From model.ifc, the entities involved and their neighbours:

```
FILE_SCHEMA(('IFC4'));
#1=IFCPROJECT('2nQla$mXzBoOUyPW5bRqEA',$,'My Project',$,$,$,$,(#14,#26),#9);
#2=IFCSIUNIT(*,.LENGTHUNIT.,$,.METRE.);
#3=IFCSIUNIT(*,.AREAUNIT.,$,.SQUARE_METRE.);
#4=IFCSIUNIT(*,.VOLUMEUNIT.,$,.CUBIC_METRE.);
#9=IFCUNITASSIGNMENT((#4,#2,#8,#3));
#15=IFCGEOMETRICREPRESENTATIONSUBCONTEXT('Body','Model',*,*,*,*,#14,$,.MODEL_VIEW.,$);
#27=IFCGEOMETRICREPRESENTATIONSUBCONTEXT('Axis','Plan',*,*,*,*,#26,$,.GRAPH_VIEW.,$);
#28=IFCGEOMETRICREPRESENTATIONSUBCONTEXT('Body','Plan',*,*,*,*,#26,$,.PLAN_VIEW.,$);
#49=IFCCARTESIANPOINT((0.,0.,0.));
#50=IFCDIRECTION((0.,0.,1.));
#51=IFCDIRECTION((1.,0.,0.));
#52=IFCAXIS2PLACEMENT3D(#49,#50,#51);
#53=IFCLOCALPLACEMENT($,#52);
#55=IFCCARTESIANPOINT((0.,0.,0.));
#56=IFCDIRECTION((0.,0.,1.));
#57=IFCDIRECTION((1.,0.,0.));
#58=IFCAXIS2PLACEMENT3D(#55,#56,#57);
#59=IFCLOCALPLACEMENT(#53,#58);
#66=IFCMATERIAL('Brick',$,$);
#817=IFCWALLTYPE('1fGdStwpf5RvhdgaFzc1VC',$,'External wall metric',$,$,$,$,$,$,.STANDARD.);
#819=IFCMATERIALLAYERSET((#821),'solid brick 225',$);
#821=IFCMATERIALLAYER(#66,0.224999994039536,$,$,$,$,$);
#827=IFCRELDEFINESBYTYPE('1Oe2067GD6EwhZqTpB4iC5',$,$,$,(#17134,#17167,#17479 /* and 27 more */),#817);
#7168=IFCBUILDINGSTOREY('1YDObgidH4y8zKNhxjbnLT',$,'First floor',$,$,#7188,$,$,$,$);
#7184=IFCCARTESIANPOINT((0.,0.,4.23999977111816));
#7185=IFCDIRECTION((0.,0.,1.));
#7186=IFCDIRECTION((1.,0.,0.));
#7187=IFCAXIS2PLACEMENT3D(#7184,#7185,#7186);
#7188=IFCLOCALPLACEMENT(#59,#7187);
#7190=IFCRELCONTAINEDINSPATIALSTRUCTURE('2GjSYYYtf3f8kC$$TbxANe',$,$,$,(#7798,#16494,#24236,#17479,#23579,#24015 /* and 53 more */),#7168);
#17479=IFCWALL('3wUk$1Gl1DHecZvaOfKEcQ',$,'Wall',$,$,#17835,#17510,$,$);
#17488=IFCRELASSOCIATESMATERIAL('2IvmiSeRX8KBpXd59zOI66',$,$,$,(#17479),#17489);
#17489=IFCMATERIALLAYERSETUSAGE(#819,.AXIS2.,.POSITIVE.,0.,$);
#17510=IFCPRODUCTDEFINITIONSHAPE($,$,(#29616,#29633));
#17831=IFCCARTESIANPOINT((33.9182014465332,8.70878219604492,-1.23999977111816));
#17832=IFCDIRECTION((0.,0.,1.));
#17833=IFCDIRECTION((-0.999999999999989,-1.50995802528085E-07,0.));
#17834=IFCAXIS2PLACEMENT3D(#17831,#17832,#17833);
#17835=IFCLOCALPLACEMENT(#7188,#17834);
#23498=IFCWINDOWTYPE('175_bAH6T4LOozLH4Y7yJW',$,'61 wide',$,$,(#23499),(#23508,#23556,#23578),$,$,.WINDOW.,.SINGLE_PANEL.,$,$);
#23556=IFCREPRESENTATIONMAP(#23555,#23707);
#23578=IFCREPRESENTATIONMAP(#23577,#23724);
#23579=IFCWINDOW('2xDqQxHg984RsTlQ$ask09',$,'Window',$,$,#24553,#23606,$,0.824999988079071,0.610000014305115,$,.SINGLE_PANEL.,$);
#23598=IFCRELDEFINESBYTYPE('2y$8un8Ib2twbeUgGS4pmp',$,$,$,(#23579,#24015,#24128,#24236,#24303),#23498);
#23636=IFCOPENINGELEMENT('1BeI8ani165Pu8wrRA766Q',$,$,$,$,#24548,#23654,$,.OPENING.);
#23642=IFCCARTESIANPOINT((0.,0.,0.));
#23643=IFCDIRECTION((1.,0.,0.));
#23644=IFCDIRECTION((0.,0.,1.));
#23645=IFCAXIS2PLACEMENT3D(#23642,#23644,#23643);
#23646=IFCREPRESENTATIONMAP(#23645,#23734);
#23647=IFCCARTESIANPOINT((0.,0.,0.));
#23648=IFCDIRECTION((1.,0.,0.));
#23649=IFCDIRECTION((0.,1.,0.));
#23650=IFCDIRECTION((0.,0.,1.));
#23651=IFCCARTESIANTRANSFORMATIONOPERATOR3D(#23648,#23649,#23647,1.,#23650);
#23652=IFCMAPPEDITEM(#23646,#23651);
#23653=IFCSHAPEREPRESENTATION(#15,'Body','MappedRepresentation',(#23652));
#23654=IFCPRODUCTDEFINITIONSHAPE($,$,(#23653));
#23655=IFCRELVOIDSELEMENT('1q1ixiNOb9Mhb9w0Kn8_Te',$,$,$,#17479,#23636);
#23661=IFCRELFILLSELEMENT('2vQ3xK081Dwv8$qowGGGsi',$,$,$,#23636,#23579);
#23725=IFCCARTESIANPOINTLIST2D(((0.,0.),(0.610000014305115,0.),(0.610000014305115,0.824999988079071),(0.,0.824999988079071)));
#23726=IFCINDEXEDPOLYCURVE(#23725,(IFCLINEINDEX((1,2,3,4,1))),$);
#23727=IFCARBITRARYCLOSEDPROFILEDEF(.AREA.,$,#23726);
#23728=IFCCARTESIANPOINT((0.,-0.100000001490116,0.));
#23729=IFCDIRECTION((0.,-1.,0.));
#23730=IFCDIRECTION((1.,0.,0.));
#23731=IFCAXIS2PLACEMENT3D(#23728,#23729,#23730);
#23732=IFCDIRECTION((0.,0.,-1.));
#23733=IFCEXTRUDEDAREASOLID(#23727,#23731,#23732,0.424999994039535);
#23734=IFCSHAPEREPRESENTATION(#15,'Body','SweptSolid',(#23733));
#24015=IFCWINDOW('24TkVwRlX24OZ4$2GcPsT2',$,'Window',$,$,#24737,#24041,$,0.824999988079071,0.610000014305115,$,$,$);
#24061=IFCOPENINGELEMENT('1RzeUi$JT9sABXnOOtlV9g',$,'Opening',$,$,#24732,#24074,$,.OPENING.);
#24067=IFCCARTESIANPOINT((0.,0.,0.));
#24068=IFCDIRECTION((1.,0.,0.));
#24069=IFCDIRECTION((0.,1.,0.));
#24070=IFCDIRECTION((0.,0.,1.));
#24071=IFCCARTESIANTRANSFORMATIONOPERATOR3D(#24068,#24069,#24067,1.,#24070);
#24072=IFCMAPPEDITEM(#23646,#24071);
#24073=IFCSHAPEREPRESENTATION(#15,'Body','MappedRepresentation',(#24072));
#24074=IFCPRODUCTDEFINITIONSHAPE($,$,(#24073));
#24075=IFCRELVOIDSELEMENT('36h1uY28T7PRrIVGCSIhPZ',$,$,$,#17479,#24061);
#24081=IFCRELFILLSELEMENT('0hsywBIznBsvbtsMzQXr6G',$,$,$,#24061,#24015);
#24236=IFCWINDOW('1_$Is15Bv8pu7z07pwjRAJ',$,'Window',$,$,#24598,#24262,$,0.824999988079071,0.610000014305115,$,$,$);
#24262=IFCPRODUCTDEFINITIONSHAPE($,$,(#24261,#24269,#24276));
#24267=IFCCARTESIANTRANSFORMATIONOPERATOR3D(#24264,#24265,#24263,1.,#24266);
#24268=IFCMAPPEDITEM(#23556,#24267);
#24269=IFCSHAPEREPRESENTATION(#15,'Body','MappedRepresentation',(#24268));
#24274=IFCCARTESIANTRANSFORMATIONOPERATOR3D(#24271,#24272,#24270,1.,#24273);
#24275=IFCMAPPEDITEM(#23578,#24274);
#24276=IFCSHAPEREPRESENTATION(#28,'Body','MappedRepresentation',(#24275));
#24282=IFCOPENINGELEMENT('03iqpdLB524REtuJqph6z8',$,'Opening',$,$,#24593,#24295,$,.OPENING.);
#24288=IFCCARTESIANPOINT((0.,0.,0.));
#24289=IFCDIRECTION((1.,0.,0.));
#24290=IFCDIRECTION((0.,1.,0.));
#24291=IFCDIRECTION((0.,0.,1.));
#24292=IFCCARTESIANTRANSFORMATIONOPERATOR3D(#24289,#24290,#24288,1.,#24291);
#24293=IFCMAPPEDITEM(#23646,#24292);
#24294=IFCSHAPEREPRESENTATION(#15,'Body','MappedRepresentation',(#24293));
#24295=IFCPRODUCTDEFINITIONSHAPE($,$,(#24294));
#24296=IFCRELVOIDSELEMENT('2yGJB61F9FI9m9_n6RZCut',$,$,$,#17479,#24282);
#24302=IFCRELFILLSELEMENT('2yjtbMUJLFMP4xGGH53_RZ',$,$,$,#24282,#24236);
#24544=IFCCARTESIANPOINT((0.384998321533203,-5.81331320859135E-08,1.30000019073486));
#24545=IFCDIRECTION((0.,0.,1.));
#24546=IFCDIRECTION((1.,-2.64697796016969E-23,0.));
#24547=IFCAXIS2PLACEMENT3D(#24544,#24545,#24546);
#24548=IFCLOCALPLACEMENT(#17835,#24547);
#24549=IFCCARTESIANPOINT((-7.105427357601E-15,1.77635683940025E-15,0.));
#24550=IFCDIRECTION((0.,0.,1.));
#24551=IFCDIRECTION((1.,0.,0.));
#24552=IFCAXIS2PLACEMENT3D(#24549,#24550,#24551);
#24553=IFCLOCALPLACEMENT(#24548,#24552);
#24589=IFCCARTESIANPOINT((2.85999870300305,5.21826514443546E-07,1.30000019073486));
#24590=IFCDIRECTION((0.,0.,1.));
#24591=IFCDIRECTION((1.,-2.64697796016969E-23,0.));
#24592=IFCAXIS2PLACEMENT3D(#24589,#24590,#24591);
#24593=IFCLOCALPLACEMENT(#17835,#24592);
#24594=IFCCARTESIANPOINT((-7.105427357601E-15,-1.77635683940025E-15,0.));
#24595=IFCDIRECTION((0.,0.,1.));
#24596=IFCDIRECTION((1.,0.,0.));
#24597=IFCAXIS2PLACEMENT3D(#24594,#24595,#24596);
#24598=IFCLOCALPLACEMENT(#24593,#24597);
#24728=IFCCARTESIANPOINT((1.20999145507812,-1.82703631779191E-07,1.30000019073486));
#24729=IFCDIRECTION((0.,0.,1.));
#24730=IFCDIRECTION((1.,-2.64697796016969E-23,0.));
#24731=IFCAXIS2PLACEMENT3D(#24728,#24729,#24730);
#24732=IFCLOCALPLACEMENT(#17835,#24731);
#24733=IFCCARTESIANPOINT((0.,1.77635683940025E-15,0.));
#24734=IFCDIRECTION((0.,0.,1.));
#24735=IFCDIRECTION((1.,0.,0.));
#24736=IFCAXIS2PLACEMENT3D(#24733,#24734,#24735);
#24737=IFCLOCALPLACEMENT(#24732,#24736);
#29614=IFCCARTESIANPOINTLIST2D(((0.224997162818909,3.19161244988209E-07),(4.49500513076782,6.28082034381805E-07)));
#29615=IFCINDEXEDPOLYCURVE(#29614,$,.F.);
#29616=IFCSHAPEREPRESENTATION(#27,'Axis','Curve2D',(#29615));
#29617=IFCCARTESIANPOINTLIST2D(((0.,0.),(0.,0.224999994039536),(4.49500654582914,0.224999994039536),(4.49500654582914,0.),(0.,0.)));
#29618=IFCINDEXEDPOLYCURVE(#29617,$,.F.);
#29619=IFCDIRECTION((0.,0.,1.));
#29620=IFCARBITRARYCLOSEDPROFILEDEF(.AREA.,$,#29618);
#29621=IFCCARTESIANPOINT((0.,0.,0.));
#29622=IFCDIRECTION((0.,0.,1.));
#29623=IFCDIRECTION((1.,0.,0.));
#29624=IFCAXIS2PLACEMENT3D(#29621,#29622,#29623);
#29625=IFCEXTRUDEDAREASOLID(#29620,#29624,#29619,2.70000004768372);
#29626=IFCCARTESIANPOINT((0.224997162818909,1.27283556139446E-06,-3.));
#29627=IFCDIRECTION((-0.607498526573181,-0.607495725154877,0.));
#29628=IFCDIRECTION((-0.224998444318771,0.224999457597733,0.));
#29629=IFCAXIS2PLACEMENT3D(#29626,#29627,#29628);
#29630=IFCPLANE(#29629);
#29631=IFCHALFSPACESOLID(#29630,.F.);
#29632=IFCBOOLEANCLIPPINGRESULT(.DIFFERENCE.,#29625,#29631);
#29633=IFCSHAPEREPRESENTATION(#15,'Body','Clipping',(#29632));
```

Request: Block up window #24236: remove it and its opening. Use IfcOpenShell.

```python
import ifcopenshell
import ifcopenshell.api.feature
import ifcopenshell.api.root
import ifcopenshell.geom
import ifcopenshell.util.shape

model = ifcopenshell.open("model.ifc")
settings = ifcopenshell.geom.settings()


def volume(element):
    """Net volume in cubic metres, openings subtracted."""
    shape = ifcopenshell.geom.create_shape(settings, element)
    return ifcopenshell.util.shape.get_volume(shape.geometry)


window = model.by_guid("1_$Is15Bv8pu7z07pwjRAJ")
opening = window.FillsVoids[0].RelatingOpeningElement
wall = opening.VoidsElements[0].RelatingBuildingElement
before = volume(wall)

ifcopenshell.api.root.remove_product(model, product=window)
ifcopenshell.api.feature.remove_feature(model, feature=opening)

after = volume(wall)

print(f"wall volume {before:.3f} -> {after:.3f} m3")

model.write("model_rev.ifc")
```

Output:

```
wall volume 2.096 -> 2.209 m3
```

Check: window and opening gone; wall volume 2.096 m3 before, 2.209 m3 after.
